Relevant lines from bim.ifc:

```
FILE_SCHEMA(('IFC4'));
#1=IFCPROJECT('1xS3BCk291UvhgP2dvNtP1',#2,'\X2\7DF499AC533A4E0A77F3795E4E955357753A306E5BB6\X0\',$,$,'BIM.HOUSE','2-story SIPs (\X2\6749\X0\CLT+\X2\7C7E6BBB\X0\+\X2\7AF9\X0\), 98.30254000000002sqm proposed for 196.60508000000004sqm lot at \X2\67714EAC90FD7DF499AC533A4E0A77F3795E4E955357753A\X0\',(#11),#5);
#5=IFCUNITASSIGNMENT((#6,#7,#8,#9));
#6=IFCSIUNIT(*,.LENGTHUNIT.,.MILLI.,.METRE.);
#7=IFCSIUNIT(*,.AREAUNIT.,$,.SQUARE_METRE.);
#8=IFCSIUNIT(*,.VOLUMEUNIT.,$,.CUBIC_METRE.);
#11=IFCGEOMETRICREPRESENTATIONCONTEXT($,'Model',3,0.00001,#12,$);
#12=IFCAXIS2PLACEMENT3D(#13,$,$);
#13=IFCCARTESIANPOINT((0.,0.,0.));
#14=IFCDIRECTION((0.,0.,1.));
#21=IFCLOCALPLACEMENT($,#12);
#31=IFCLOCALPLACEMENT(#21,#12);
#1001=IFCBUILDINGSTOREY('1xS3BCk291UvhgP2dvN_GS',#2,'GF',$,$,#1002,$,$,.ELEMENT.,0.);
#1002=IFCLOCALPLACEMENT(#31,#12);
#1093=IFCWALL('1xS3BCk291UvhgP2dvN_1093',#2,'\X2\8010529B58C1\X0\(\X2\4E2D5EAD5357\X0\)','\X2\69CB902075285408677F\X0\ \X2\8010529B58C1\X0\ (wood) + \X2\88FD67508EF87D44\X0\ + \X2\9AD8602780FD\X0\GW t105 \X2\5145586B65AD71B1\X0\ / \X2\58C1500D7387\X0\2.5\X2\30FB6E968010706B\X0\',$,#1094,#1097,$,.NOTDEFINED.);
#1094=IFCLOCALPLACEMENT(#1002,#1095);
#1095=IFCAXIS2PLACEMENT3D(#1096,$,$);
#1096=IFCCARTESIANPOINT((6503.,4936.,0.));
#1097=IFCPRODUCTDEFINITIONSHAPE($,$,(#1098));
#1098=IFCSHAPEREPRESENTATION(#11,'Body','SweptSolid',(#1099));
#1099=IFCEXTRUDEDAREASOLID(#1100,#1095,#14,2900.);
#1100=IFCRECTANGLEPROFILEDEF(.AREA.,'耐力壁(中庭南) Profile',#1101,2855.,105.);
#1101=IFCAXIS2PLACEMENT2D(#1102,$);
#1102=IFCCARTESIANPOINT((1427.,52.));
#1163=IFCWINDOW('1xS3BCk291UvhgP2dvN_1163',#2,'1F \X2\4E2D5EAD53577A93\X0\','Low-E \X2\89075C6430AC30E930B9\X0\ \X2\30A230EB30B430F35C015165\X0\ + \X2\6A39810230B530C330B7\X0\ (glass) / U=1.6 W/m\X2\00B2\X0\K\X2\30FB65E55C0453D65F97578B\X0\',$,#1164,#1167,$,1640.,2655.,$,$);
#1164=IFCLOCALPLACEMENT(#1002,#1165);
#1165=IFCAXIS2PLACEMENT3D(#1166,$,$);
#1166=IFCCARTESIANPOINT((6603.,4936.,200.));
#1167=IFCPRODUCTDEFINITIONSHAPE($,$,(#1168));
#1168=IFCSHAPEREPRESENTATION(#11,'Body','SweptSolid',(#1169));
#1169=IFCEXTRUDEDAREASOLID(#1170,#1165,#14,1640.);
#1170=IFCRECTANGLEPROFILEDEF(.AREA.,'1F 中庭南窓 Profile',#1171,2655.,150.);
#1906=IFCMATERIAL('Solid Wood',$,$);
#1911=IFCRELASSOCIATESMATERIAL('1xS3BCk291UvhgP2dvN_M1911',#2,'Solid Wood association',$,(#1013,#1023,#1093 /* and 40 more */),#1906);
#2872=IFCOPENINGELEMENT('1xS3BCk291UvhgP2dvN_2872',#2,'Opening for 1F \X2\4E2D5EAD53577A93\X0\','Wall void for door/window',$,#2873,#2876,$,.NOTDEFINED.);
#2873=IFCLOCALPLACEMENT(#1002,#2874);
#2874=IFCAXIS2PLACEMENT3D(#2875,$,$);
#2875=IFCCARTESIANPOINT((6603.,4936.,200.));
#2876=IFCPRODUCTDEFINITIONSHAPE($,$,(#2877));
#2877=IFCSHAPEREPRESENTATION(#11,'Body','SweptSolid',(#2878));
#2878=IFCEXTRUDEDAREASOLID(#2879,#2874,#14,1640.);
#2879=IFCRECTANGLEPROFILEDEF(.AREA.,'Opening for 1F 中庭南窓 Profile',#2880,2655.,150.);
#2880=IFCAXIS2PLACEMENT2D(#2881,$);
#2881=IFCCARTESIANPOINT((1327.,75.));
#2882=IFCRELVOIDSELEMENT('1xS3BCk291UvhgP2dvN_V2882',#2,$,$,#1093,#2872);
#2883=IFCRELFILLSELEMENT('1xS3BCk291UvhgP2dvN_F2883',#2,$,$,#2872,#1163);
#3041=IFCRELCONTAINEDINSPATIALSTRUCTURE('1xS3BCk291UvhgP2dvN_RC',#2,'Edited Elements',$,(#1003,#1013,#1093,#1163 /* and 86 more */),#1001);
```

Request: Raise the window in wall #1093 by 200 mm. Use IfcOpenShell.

```python
import numpy as np
import ifcopenshell
import ifcopenshell.api.geometry
import ifcopenshell.util.placement
import ifcopenshell.util.unit

model = ifcopenshell.open("bim.ifc")
unit_scale = ifcopenshell.util.unit.calculate_unit_scale(model)

window = model.by_guid("1xS3BCk291UvhgP2dvN_1163")
opening = window.FillsVoids[0].RelatingOpeningElement
dz = 200.0

shift = np.array([0.0, 0.0, dz])
# The window is not placed relative to its opening, so move both.
for product in (opening, window):
    matrix = ifcopenshell.util.placement.get_local_placement(product.ObjectPlacement)
    matrix[:3, 3] += shift
    ifcopenshell.api.geometry.edit_object_placement(model, product=product, matrix=matrix, is_si=False)

print(f"moved by {dz * unit_scale:+.3f} m")

model.write("bim-out.ifc")
```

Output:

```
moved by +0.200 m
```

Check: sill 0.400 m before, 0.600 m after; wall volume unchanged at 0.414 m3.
